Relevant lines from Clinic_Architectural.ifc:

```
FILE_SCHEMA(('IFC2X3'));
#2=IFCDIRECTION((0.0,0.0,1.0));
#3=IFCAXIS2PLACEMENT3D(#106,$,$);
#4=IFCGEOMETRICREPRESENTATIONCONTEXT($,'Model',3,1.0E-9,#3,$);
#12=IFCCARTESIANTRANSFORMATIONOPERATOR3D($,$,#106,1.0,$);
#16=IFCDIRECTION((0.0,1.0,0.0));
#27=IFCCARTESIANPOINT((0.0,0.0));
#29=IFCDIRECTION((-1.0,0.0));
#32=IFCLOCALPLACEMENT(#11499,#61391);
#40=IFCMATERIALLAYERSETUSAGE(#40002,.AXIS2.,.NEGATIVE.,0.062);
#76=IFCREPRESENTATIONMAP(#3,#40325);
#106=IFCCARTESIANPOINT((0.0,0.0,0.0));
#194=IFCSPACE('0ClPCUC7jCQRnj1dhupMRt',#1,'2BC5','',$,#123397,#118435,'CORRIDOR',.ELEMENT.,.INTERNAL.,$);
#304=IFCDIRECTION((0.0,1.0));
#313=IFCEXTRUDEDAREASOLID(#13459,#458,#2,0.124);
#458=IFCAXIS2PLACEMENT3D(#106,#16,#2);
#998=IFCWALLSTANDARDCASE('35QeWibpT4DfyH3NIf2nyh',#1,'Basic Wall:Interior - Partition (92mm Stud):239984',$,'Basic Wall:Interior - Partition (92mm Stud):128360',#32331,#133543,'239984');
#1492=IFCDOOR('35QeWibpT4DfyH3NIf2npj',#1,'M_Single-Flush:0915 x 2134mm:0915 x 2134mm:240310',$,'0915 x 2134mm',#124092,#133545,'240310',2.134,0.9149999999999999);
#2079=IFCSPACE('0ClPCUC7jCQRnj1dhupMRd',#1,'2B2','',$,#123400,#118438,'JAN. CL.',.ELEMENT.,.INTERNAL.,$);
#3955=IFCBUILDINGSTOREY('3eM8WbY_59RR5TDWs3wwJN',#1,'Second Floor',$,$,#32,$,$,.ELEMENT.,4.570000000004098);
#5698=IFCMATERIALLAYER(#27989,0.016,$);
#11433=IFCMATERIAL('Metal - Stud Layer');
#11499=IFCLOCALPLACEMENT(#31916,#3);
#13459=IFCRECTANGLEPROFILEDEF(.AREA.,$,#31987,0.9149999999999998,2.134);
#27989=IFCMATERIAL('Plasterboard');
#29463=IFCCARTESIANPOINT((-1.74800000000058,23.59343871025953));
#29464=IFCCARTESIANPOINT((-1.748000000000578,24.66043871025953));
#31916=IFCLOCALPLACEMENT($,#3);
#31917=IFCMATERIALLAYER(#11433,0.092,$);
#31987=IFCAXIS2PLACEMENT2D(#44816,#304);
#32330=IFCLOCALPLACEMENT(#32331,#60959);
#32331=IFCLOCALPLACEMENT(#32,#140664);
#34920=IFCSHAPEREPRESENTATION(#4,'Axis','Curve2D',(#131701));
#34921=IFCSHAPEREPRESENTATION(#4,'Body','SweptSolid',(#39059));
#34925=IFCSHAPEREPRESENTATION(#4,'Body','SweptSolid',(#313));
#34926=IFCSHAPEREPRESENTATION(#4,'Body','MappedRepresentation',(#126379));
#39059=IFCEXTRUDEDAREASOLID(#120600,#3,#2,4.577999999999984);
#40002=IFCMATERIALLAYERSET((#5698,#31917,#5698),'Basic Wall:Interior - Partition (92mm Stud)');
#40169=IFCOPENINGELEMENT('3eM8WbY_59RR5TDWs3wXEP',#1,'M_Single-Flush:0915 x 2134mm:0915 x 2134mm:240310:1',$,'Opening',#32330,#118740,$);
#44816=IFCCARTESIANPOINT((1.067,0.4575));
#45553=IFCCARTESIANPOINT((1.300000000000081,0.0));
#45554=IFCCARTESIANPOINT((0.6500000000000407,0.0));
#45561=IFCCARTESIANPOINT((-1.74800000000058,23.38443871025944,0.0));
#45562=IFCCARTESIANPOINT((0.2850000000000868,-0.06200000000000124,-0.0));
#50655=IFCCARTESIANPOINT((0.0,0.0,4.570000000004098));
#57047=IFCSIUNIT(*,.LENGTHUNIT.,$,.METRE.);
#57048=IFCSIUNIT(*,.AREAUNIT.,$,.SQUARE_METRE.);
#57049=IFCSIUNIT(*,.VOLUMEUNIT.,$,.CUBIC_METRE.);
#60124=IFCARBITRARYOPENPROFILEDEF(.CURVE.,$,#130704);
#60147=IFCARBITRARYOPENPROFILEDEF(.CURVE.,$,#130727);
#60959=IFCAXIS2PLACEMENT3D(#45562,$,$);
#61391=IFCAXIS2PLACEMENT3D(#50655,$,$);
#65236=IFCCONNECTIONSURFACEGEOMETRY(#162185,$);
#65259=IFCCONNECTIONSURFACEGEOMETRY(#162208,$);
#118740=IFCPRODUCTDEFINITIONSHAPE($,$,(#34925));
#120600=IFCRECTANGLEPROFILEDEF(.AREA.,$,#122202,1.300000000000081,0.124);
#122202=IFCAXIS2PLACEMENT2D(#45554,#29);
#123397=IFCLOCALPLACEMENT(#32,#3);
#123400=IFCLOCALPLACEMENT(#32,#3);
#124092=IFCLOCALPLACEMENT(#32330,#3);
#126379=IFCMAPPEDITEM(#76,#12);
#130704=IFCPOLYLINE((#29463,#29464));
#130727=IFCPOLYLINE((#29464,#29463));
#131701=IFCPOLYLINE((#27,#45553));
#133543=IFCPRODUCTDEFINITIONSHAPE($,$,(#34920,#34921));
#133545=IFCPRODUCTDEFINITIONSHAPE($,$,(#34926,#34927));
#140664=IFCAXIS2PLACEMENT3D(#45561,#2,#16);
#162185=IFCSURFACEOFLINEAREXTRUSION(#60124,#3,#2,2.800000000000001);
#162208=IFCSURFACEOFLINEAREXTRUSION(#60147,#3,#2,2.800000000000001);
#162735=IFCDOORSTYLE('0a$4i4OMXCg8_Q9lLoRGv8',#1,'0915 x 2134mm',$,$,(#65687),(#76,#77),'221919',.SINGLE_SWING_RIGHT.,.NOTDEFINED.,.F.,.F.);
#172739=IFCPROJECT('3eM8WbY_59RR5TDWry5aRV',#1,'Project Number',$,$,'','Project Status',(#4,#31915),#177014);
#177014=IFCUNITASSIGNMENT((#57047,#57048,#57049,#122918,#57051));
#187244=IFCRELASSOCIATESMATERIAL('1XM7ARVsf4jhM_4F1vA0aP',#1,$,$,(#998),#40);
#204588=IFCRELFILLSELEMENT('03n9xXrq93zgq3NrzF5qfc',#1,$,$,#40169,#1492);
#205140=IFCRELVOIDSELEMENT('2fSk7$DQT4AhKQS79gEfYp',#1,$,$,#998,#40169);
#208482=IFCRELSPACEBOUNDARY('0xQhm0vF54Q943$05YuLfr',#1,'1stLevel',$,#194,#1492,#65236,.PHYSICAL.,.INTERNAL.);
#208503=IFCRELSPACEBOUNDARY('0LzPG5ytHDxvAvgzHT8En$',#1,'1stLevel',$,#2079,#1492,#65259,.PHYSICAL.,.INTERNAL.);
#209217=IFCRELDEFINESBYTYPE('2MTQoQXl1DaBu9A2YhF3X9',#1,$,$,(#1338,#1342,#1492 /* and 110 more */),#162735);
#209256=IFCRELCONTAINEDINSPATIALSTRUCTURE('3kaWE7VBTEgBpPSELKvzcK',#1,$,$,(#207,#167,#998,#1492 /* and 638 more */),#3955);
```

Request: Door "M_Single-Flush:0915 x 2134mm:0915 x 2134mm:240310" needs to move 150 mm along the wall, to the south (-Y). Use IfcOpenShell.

```python
import numpy as np
import ifcopenshell
import ifcopenshell.api.geometry
import ifcopenshell.util.placement
import ifcopenshell.util.unit

model = ifcopenshell.open("Clinic_Architectural.ifc")
unit_scale = ifcopenshell.util.unit.calculate_unit_scale(model)

door = model.by_id(1492)
opening = door.FillsVoids[0].RelatingOpeningElement
wall = opening.VoidsElements[0].RelatingBuildingElement

wall_matrix = ifcopenshell.util.placement.get_local_placement(wall.ObjectPlacement)
shift = wall_matrix[:3, 0] * -0.15 / unit_scale
before = ifcopenshell.util.placement.get_local_placement(door.ObjectPlacement)[:3, 3].copy()

# The door is placed relative to its opening, so it follows when the opening moves.
matrix = ifcopenshell.util.placement.get_local_placement(opening.ObjectPlacement)
matrix[:3, 3] += shift
ifcopenshell.api.geometry.edit_object_placement(
    model, product=opening, matrix=matrix, is_si=False, should_transform_children=True
)

# Space boundary surfaces are stored in each space's coordinates; move them too.
for rel in door.ProvidesBoundaries:
    if not rel.ConnectionGeometry:
        continue
    surface = rel.ConnectionGeometry.SurfaceOnRelatingElement
    space_matrix = ifcopenshell.util.placement.get_local_placement(rel.RelatingSpace.ObjectPlacement)
    point = np.array(surface.Position.Location.Coordinates) + space_matrix[:3, :3].T @ shift
    surface.Position = model.createIfcAxis2Placement3D(
        model.createIfcCartesianPoint(point.tolist()), surface.Position.Axis, surface.Position.RefDirection
    )

after = ifcopenshell.util.placement.get_local_placement(door.ObjectPlacement)[:3, 3]
print("door moved by", (after - before).round(3) + 0.0)

model.write("Clinic_Architectural_rev.ifc")
```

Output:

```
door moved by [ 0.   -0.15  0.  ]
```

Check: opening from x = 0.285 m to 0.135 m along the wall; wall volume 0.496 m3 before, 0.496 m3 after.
